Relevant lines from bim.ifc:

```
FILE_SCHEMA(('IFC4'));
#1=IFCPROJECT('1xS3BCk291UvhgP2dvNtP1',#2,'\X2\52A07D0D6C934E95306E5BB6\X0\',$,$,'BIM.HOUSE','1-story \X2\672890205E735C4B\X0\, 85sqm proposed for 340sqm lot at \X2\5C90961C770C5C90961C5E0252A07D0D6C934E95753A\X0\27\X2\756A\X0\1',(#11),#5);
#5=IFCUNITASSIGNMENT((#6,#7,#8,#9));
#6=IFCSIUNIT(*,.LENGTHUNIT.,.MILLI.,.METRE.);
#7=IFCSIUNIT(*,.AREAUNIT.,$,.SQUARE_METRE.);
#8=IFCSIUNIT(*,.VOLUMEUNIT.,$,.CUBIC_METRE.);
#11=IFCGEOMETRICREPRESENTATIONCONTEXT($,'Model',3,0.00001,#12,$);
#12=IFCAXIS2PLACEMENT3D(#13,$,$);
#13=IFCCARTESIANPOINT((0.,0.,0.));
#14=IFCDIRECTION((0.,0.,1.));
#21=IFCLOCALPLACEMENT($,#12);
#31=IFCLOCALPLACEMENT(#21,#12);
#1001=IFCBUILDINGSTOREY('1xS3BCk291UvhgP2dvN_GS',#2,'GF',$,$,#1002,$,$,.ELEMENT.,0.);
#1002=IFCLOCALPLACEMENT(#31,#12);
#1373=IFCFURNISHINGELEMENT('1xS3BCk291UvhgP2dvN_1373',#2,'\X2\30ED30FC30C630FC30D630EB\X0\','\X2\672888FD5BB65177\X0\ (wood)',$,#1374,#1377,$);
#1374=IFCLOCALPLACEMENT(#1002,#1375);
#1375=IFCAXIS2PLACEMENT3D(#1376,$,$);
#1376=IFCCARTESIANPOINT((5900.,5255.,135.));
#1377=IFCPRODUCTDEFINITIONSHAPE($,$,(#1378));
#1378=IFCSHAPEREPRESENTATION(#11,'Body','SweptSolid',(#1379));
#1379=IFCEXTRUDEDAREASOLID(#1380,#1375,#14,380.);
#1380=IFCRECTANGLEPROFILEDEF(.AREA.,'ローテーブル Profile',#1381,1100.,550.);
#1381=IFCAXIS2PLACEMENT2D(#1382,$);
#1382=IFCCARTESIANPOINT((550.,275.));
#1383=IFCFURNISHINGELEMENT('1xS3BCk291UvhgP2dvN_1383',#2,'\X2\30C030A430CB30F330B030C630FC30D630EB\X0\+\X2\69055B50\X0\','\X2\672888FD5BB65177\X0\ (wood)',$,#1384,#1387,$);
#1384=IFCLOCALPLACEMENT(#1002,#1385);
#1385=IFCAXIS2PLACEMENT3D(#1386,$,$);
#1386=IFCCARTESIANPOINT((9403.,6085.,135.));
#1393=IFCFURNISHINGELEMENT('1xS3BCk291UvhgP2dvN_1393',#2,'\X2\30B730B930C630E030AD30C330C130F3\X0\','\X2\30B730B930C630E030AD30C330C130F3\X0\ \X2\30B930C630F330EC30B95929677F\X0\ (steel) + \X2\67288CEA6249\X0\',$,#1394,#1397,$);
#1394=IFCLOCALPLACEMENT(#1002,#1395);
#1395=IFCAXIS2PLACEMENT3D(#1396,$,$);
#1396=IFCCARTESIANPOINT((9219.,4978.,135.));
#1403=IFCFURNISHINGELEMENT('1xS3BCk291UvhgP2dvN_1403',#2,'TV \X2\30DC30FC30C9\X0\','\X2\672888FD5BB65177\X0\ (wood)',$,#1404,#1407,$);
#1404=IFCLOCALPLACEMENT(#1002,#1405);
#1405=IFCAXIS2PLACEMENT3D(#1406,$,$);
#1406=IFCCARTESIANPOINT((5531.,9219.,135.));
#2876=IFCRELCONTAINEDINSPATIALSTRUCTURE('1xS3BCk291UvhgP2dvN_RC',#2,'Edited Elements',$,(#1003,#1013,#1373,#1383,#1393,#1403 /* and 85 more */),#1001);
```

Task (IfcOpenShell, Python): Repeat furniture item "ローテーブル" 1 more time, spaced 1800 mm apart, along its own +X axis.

```python
import ifcopenshell
import ifcopenshell.api.geometry
import ifcopenshell.api.root
import ifcopenshell.util.element
import ifcopenshell.util.placement
import ifcopenshell.util.unit

model = ifcopenshell.open("bim.ifc")
unit_scale = ifcopenshell.util.unit.calculate_unit_scale(model)


def reuse_history(source, copy):
    """copy_class also copies each property set's owner history, people and application; keep the originals."""
    for rel in copy.IsDefinedBy:
        if rel.is_a("IfcRelDefinesByProperties") and (history := rel.RelatingPropertyDefinition.OwnerHistory):
            rel.RelatingPropertyDefinition.OwnerHistory = source.OwnerHistory
            ifcopenshell.util.element.remove_deep2(model, history)


source = model.by_guid("1xS3BCk291UvhgP2dvN_1373")
base = ifcopenshell.util.placement.get_local_placement(source.ObjectPlacement)
step = base[:3, 0] * 1.8 / unit_scale

for i in range(1, 2):
    copy = ifcopenshell.api.root.copy_class(model, product=source)
    copy.Representation = ifcopenshell.util.element.copy_deep(
        model, source.Representation, exclude=["IfcGeometricRepresentationContext", "IfcRepresentationMap"]
    )
    reuse_history(source, copy)
    matrix = base.copy()
    matrix[:3, 3] += i * step
    print("added at", matrix[:3, 3].round(3) + 0.0)
    ifcopenshell.api.geometry.edit_object_placement(model, product=copy, matrix=matrix, is_si=False)

model.write("bim_v2.ifc")
```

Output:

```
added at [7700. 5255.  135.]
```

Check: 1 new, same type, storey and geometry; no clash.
